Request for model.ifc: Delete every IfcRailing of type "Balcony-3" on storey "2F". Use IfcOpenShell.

First a look at what the model holds.

```python
import ifcopenshell
import ifcopenshell.util.element

model = ifcopenshell.open("model.ifc")
print(model.schema)
storey = next(s for s in model.by_type("IfcBuildingStorey") if s.Name == "2F")
railings = [e for e in ifcopenshell.util.element.get_decomposition(storey) if e.is_a("IfcRailing")]
seen = {}
for e in railings:
    element_type = ifcopenshell.util.element.get_type(e)
    name = element_type.Name if element_type not in (None, e) else None
    seen[name] = seen.get(name, 0) + 1
for name, count in sorted(seen.items(), key=str):
    print(count, "x", name)
```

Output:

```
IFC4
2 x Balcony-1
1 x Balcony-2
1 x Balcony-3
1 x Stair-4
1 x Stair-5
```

```python
import ifcopenshell
import ifcopenshell.api.root
import ifcopenshell.util.element

model = ifcopenshell.open("model.ifc")

storey = next(s for s in model.by_type("IfcBuildingStorey") if s.Name == "2F")
railings = [e for e in ifcopenshell.util.element.get_decomposition(storey) if e.is_a("IfcRailing")]
targets = [e for e in railings if (t := ifcopenshell.util.element.get_type(e)) not in (None, e) and t.Name == "Balcony-3"]

for e in targets:
    ifcopenshell.api.root.remove_product(model, product=e)
print(len(targets), "removed")

model.write("model_rev.ifc")
```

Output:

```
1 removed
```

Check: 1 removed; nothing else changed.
